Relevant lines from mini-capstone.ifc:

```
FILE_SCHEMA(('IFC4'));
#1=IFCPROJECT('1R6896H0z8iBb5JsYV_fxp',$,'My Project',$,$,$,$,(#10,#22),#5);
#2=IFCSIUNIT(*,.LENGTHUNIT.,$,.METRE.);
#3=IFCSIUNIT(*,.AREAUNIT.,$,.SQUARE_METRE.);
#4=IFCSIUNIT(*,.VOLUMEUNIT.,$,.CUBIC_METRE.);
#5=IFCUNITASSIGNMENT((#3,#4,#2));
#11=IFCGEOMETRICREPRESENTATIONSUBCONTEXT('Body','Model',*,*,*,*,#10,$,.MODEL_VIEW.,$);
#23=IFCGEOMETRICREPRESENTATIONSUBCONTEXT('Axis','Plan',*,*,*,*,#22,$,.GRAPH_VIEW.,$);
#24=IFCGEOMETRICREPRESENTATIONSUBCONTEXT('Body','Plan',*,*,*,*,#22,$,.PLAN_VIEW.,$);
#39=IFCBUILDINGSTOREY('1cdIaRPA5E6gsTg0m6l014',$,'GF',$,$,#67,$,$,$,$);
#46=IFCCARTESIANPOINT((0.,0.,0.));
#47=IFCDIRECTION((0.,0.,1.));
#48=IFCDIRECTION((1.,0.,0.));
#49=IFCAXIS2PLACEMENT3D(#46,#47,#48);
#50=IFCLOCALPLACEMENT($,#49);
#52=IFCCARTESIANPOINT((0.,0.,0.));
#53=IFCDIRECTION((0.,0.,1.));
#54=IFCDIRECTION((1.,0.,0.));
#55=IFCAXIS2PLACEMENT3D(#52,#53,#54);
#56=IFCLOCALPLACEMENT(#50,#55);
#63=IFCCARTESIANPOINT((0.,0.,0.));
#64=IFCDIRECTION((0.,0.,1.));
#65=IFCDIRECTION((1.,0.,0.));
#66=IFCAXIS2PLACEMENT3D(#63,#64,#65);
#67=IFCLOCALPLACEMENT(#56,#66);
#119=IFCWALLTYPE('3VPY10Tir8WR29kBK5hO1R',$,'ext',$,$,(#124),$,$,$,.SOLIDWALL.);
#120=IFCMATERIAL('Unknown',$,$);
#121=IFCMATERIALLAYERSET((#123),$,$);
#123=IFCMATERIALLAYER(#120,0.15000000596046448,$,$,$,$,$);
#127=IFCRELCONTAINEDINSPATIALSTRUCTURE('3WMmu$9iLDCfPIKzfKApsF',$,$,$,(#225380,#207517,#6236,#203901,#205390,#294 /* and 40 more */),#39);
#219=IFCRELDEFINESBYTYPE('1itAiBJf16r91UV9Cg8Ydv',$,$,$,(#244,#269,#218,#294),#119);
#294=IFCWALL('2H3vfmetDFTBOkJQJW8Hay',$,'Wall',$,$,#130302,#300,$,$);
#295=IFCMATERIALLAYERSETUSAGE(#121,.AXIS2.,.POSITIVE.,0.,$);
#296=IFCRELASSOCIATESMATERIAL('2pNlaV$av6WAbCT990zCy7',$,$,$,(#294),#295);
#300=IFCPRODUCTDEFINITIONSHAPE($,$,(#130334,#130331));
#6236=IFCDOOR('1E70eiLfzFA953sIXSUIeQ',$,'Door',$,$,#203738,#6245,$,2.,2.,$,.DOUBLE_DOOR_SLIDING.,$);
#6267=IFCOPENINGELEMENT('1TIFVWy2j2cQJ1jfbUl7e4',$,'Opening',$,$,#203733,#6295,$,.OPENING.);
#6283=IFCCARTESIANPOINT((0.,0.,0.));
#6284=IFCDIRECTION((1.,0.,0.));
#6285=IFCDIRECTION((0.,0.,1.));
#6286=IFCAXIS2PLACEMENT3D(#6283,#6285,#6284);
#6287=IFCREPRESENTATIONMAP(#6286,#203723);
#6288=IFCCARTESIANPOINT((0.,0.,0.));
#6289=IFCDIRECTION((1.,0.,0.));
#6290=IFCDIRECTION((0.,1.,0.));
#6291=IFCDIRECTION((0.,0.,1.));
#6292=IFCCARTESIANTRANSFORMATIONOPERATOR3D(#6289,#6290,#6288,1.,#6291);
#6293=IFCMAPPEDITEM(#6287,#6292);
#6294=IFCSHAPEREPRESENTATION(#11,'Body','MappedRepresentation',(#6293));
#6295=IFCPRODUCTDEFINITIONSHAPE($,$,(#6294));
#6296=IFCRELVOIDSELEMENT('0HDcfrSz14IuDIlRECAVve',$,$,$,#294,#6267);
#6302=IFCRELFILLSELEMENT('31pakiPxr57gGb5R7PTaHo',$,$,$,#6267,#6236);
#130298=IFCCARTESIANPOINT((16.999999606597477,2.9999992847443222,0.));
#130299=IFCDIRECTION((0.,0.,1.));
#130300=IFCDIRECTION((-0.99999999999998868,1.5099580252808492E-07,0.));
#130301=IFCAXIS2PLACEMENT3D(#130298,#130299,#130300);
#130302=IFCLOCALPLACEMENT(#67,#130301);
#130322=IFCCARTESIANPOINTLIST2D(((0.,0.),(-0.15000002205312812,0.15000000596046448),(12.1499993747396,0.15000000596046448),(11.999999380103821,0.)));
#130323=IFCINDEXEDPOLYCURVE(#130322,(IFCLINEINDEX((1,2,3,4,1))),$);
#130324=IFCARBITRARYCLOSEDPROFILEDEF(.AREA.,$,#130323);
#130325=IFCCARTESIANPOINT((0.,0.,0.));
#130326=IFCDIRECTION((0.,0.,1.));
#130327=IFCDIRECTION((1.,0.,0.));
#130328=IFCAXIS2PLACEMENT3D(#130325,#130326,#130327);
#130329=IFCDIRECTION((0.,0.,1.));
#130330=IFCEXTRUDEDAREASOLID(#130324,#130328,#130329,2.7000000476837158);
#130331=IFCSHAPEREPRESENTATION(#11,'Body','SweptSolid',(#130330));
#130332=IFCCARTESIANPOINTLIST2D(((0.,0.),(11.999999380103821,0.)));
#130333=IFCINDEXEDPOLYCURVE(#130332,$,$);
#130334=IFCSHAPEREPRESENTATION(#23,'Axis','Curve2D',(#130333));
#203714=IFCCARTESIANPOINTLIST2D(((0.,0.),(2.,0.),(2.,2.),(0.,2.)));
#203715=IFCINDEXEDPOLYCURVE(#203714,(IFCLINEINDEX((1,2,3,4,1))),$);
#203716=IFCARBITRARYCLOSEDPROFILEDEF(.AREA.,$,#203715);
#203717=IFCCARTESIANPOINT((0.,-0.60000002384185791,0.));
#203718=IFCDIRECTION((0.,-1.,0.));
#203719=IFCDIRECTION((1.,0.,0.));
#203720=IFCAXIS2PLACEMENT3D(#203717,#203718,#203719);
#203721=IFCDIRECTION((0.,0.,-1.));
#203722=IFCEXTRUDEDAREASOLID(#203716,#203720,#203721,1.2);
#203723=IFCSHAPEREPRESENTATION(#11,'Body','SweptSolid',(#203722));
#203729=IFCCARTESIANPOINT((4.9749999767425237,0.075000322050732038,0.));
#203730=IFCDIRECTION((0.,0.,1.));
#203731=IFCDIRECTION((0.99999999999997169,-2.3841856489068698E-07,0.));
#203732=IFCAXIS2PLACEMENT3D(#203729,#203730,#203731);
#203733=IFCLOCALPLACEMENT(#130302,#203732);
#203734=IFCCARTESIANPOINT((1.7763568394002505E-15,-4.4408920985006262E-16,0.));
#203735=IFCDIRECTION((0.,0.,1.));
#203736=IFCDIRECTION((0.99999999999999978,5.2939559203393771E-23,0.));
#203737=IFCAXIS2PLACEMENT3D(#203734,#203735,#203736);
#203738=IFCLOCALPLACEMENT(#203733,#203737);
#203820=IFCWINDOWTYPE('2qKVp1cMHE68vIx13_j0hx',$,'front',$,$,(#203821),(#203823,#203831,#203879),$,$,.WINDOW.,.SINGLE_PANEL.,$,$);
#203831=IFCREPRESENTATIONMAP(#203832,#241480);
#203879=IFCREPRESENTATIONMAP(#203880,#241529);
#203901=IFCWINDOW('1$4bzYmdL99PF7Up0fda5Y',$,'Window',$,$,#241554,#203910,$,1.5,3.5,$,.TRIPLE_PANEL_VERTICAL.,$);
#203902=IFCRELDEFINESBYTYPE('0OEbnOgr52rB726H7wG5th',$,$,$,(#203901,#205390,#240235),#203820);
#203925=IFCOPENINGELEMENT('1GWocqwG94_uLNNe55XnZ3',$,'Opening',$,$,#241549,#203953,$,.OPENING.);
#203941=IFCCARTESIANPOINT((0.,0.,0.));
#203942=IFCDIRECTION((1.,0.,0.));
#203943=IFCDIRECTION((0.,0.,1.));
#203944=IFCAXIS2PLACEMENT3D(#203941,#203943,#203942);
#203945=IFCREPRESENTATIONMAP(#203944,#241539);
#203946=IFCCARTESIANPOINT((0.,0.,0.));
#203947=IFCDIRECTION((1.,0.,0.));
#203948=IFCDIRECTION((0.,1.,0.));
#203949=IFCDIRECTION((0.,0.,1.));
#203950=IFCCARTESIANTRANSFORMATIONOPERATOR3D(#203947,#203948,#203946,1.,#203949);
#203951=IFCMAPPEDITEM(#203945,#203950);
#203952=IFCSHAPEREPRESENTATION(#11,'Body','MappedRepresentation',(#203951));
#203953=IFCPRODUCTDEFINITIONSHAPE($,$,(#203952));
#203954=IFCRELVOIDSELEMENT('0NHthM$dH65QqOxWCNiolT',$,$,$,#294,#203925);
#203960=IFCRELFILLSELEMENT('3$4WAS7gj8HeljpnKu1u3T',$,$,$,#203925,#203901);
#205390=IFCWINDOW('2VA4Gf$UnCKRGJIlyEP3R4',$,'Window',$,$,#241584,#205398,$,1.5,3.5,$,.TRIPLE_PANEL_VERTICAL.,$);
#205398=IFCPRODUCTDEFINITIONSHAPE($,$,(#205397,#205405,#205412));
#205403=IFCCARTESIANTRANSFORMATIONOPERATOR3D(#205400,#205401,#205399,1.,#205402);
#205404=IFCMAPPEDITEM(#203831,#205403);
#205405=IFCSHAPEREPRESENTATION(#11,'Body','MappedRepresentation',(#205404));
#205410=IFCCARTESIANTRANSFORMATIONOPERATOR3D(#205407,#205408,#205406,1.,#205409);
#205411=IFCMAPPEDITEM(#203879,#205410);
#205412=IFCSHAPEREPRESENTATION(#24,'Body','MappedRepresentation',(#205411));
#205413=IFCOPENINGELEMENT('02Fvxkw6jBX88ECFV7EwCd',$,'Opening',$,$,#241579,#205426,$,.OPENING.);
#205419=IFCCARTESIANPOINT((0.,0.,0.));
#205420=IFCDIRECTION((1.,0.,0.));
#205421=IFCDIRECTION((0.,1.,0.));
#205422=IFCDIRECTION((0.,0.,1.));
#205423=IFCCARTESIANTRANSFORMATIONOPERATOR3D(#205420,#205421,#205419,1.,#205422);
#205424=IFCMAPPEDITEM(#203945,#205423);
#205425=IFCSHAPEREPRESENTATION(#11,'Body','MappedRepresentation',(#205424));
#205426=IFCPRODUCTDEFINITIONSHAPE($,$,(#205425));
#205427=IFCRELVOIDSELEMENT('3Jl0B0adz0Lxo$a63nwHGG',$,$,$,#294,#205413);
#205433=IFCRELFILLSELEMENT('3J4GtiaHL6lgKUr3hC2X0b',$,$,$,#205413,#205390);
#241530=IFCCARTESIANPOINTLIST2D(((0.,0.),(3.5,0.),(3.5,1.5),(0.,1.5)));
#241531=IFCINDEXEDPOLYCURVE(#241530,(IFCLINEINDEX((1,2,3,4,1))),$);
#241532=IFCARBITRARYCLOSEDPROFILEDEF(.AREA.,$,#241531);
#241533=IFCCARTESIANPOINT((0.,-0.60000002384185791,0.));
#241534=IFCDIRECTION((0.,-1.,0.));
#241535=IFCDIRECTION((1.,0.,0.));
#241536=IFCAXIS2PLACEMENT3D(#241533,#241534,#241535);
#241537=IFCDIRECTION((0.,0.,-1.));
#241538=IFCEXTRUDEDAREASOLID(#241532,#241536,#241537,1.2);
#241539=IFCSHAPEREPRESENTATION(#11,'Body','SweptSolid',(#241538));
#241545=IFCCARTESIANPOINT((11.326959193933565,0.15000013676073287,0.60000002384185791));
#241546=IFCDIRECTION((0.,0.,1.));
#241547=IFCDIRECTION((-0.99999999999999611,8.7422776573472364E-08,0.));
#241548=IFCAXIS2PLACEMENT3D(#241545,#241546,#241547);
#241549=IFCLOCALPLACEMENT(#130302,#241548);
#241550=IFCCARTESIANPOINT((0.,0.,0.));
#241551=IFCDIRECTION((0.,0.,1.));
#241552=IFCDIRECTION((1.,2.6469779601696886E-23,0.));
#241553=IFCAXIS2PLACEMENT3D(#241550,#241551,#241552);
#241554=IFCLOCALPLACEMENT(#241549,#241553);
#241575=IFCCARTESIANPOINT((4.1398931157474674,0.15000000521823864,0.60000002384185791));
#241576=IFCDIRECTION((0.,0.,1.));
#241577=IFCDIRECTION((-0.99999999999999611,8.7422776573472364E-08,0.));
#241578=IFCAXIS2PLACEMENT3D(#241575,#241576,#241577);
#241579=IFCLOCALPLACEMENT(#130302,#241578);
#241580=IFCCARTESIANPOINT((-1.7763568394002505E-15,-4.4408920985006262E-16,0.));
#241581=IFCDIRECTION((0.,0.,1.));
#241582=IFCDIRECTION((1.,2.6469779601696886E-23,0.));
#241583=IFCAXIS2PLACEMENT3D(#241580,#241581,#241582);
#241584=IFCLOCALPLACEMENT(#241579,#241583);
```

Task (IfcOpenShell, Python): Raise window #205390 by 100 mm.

```python
import numpy as np
import ifcopenshell
import ifcopenshell.api.geometry
import ifcopenshell.util.placement
import ifcopenshell.util.unit

model = ifcopenshell.open("mini-capstone.ifc")
unit_scale = ifcopenshell.util.unit.calculate_unit_scale(model)

window = model.by_guid("2VA4Gf$UnCKRGJIlyEP3R4")
opening = window.FillsVoids[0].RelatingOpeningElement
dz = 0.1

shift = np.array([0.0, 0.0, dz])
# The window is placed relative to its opening, so it follows when the opening moves.
matrix = ifcopenshell.util.placement.get_local_placement(opening.ObjectPlacement)
matrix[:3, 3] += shift
ifcopenshell.api.geometry.edit_object_placement(
    model, product=opening, matrix=matrix, is_si=False, should_transform_children=True
)

print(f"moved by {dz * unit_scale:+.3f} m")

model.write("mini-capstone_rev.ifc")
```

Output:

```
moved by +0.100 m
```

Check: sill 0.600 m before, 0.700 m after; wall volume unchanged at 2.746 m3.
